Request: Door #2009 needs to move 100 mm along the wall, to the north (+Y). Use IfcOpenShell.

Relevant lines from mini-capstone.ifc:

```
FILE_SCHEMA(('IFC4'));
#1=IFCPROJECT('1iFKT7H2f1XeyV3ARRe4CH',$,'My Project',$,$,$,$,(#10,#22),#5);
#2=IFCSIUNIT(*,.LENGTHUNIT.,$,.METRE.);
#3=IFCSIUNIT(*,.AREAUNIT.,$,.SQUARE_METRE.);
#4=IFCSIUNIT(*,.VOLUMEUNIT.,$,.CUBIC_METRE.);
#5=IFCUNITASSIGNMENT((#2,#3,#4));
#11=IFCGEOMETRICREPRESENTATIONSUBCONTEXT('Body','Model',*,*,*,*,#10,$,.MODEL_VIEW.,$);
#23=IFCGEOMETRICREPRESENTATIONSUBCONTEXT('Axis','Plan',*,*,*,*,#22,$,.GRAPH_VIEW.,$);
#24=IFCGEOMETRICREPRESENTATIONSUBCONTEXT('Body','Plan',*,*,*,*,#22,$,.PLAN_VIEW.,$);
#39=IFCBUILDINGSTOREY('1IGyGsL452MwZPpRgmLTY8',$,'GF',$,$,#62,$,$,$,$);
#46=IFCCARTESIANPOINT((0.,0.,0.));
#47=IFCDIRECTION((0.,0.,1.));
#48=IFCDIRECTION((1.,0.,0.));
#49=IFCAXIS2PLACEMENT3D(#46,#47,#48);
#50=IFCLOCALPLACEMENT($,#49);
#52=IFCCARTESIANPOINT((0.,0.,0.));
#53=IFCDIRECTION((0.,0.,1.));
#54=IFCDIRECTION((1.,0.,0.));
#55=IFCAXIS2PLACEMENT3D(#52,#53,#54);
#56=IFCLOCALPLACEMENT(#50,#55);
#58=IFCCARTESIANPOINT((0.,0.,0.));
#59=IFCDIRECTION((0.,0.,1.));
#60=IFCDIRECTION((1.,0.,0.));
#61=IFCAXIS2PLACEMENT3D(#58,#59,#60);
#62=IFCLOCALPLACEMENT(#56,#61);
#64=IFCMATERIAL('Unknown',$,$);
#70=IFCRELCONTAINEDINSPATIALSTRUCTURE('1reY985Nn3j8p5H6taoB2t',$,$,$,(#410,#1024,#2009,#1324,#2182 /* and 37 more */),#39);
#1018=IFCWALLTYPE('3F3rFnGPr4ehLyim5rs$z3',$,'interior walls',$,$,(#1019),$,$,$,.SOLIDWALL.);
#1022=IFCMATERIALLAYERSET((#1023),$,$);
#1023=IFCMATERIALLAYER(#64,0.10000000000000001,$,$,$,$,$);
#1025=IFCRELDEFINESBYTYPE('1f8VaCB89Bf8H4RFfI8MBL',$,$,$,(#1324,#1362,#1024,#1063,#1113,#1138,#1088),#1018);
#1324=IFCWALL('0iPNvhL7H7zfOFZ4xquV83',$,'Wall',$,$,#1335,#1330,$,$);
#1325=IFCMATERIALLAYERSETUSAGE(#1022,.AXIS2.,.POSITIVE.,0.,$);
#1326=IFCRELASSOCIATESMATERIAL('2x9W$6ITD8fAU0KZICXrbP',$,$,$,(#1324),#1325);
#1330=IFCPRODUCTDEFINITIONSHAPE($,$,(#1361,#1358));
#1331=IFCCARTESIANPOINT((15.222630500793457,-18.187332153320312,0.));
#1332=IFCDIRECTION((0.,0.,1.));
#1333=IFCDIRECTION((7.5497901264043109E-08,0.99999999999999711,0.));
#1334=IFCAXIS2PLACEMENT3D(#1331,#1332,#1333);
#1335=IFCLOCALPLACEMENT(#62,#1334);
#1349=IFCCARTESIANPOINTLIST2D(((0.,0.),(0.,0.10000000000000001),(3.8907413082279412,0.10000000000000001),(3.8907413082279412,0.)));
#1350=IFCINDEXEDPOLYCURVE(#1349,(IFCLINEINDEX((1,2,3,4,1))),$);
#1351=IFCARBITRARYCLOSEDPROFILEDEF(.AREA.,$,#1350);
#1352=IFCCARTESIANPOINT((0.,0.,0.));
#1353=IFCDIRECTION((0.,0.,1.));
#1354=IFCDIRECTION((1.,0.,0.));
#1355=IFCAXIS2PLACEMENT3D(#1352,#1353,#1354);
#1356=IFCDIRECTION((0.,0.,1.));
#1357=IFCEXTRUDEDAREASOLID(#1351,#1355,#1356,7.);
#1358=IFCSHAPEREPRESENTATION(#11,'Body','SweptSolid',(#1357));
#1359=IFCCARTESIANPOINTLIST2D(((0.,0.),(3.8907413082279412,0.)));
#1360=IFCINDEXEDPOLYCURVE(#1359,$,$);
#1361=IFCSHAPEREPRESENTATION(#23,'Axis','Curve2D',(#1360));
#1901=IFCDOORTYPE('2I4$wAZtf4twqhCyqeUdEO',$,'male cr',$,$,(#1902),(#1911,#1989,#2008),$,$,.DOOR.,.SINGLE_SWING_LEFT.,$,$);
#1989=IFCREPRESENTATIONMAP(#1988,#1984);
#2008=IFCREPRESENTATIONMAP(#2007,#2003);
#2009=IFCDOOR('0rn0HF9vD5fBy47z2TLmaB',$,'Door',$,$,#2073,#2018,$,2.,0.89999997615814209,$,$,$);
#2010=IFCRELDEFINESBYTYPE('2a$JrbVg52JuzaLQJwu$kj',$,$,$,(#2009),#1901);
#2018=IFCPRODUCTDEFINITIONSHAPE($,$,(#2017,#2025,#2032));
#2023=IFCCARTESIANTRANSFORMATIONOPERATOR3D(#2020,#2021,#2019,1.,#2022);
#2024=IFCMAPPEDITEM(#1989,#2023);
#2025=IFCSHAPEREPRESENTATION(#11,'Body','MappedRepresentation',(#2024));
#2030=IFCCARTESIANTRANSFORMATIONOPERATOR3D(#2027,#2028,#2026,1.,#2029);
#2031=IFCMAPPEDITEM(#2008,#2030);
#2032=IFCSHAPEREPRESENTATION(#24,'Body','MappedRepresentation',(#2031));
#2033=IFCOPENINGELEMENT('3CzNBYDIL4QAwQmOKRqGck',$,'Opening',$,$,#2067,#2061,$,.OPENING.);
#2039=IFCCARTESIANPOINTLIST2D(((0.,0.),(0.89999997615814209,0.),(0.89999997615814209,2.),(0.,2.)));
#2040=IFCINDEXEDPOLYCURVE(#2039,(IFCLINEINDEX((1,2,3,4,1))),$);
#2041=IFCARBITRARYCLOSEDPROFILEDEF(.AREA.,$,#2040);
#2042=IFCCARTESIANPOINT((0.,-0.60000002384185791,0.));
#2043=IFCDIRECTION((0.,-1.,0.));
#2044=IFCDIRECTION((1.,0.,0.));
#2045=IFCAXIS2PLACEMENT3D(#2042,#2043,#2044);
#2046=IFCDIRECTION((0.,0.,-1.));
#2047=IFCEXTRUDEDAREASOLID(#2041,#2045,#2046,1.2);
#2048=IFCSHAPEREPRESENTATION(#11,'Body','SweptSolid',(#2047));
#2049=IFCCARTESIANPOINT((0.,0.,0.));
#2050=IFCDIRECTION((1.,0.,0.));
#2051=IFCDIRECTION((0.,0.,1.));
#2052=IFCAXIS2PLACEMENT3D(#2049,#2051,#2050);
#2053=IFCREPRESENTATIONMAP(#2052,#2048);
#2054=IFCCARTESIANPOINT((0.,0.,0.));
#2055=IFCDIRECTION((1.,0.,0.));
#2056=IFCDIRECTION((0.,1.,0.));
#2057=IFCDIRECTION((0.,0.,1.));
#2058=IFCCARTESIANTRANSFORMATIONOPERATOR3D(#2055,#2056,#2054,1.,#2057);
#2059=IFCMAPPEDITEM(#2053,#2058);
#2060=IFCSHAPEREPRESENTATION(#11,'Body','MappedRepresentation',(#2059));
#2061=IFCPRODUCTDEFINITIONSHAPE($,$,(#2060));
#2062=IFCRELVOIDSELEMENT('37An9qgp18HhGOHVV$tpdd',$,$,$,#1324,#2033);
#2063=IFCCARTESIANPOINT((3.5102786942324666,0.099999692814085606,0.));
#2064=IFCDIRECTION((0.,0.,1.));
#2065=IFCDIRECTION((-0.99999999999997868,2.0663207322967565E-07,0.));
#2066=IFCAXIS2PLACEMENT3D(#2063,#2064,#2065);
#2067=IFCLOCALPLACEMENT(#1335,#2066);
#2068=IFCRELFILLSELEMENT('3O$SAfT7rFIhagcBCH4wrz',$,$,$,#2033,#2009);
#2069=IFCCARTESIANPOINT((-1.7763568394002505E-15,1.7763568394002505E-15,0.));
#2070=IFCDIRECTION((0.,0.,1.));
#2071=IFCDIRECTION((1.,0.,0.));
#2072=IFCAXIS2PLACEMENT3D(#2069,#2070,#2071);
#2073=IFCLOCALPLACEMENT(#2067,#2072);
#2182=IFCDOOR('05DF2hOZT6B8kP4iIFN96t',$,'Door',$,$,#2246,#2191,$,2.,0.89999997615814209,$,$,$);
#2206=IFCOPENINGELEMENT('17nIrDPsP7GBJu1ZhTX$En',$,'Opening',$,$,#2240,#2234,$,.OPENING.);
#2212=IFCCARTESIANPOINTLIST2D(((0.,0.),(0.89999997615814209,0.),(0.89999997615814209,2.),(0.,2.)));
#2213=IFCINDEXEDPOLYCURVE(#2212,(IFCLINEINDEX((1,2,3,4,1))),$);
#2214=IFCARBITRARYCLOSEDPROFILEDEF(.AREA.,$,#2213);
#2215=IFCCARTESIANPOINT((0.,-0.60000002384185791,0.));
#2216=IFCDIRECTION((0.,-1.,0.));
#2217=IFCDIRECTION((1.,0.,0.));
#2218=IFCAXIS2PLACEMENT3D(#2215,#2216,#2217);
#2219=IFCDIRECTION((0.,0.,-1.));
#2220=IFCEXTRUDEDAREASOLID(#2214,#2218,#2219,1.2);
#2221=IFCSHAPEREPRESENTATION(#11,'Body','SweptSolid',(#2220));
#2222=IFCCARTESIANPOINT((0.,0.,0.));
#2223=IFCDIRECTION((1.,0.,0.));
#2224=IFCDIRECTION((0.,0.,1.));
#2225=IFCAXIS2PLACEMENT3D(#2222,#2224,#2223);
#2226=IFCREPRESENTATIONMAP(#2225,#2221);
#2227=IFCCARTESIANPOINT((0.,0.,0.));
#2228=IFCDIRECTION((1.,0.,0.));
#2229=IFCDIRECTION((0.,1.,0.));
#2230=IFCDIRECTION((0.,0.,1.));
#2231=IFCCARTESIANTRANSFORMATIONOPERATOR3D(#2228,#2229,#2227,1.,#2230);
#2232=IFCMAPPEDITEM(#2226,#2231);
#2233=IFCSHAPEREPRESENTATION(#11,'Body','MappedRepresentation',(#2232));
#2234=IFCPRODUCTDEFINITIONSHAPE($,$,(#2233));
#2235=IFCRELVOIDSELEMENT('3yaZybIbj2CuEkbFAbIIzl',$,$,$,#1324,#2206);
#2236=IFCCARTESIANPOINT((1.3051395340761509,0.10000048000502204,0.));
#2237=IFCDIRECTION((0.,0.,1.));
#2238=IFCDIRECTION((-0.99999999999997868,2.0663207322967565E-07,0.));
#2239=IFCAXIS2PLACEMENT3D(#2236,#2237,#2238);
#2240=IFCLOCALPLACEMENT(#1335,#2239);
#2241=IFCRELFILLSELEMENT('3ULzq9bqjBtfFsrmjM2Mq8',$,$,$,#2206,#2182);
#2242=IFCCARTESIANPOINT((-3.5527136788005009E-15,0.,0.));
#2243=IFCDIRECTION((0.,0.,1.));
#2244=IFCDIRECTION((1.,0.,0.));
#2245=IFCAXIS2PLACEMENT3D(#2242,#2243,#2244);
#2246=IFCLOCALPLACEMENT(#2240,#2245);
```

```python
import ifcopenshell
import ifcopenshell.api.geometry
import ifcopenshell.util.placement
import ifcopenshell.util.unit

model = ifcopenshell.open("mini-capstone.ifc")
unit_scale = ifcopenshell.util.unit.calculate_unit_scale(model)

door = model.by_id(2009)
opening = door.FillsVoids[0].RelatingOpeningElement
wall = opening.VoidsElements[0].RelatingBuildingElement

wall_matrix = ifcopenshell.util.placement.get_local_placement(wall.ObjectPlacement)
shift = wall_matrix[:3, 0] * 0.1 / unit_scale
before = ifcopenshell.util.placement.get_local_placement(door.ObjectPlacement)[:3, 3].copy()

# The door is placed relative to its opening, so it follows when the opening moves.
matrix = ifcopenshell.util.placement.get_local_placement(opening.ObjectPlacement)
matrix[:3, 3] += shift
ifcopenshell.api.geometry.edit_object_placement(
    model, product=opening, matrix=matrix, is_si=False, should_transform_children=True
)

after = ifcopenshell.util.placement.get_local_placement(door.ObjectPlacement)[:3, 3]
print("door moved by", (after - before).round(3) + 0.0)

model.write("mini-capstone_edited.ifc")
```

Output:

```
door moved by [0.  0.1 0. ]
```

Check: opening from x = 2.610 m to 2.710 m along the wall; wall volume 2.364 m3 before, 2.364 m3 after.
